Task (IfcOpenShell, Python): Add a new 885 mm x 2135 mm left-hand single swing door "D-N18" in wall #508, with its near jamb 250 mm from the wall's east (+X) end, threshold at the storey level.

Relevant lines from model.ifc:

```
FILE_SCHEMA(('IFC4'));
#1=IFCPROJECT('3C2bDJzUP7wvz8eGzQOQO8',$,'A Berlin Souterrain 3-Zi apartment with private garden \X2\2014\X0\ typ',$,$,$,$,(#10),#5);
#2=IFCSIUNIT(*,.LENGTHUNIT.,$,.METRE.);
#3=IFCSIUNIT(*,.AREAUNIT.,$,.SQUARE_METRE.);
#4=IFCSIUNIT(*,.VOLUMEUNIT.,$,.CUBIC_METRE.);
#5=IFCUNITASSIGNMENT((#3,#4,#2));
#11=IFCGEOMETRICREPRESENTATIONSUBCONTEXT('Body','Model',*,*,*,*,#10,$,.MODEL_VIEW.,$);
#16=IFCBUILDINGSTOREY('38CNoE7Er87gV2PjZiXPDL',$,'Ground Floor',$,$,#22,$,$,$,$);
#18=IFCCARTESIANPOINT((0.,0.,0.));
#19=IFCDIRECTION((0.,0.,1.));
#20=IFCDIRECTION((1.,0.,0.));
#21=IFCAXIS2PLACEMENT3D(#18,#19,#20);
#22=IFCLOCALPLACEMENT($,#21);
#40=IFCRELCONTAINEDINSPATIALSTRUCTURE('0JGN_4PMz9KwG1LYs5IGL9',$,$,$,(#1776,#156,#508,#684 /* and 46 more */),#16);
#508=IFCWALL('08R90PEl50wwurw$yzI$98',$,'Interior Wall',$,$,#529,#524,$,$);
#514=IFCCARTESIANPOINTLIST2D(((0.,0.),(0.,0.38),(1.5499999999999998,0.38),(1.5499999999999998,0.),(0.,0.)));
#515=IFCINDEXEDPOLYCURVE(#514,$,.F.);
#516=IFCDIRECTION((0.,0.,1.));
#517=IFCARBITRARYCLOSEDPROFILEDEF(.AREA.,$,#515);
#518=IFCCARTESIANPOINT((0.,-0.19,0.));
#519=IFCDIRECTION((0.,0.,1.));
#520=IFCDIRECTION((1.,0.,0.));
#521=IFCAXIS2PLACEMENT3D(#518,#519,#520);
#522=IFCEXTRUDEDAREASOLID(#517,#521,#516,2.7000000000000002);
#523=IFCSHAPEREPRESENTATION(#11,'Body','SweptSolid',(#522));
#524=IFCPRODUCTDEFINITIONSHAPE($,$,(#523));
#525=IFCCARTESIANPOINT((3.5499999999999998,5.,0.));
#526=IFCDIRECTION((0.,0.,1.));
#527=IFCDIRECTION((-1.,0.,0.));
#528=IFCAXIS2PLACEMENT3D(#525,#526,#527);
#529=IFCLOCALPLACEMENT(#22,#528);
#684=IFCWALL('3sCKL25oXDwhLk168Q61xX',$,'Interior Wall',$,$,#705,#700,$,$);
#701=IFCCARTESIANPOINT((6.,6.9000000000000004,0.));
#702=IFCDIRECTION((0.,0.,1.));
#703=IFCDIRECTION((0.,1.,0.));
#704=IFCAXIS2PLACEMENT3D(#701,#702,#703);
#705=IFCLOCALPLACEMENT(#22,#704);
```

```python
import numpy as np
import ifcopenshell
import ifcopenshell.api.feature
import ifcopenshell.api.geometry
import ifcopenshell.api.root
import ifcopenshell.api.spatial
import ifcopenshell.geom
import ifcopenshell.util.element
import ifcopenshell.util.placement
import ifcopenshell.util.representation
import ifcopenshell.util.shape
import ifcopenshell.util.unit

model = ifcopenshell.open("model.ifc")
unit_scale = ifcopenshell.util.unit.calculate_unit_scale(model)
settings = ifcopenshell.geom.settings()


def volume(element):
    """Net volume in cubic metres, openings subtracted."""
    shape = ifcopenshell.geom.create_shape(settings, element)
    return ifcopenshell.util.shape.get_volume(shape.geometry)


wall = model.by_guid("08R90PEl50wwurw$yzI$98")
storey = ifcopenshell.util.element.get_container(wall, ifc_class="IfcBuildingStorey")
context = ifcopenshell.util.representation.get_context(model, "Model", "Body", "MODEL_VIEW")
before = volume(wall)

width, height, from_end, sill = 0.885, 2.135, 0.25, 0.0  # metres

# The wall runs along its own X axis, and the end named is its -X end.
wall_shape = ifcopenshell.geom.create_shape(settings, wall)
x, y, z = ifcopenshell.util.shape.get_vertices(wall_shape.geometry).T
start = x.min() + from_end
face, thickness = float(y.min()), float(y.max() - y.min())
wall_matrix = ifcopenshell.util.placement.get_local_placement(wall.ObjectPlacement)
level = ifcopenshell.util.placement.get_local_placement(storey.ObjectPlacement)[2, 3]


def in_wall(x, y):
    """Placement at x, y metres in the wall's axes, at sill height."""
    matrix = wall_matrix.copy()
    matrix[:, 3] = wall_matrix @ np.array([x / unit_scale, y / unit_scale, 0.0, 1.0])
    matrix[2, 3] = level + sill / unit_scale
    return matrix


# Opening: a box that overshoots both wall faces by 50 mm.
opening = ifcopenshell.api.root.create_entity(model, ifc_class="IfcOpeningElement", predefined_type="OPENING")
box = ifcopenshell.api.geometry.add_wall_representation(
    model, context=context, length=width, height=height, thickness=thickness + 0.1
)
ifcopenshell.api.geometry.assign_representation(model, product=opening, representation=box)
ifcopenshell.api.geometry.edit_object_placement(model, product=opening, matrix=in_wall(start, face - 0.05), is_si=False)
ifcopenshell.api.feature.add_feature(model, feature=opening, element=wall)

door = ifcopenshell.api.root.create_entity(model, ifc_class="IfcDoor", name="D-N18", predefined_type="DOOR")
door.OverallWidth, door.OverallHeight = width / unit_scale, height / unit_scale
door.OperationType = "SINGLE_SWING_LEFT"
body = ifcopenshell.api.geometry.add_door_representation(
    model,
    context=context,
    overall_width=door.OverallWidth,
    overall_height=door.OverallHeight,
    operation_type="SINGLE_SWING_LEFT",
    lining_properties={"LiningDepth": thickness / unit_scale, "ThresholdDepth": thickness / unit_scale},
)
ifcopenshell.api.geometry.assign_representation(model, product=door, representation=body)
ifcopenshell.api.spatial.assign_container(model, products=[door], relating_structure=storey)
ifcopenshell.api.feature.add_filling(model, opening=opening, element=door)

# The lining spans the wall, so the door starts at the wall face.
ifcopenshell.api.geometry.edit_object_placement(model, product=door, matrix=in_wall(start, face), is_si=False)

after = volume(wall)

print(f"wall volume {before:.3f} -> {after:.3f} m3")

model.write("model_rev.ifc")
```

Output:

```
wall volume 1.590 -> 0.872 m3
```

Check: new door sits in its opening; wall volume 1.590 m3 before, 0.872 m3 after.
